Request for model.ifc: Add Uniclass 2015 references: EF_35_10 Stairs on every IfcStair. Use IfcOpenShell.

First a look at what the model holds.

```python
import ifcopenshell

model = ifcopenshell.open("model.ifc")
print(model.schema)
print("classifications:", [c.Name for c in model.by_type("IfcClassification")])
for ifc_class in ("IfcDoor", "IfcRoof", "IfcStair", "IfcWall", "IfcWindow"):
    print(ifc_class, len(model.by_type(ifc_class)))
```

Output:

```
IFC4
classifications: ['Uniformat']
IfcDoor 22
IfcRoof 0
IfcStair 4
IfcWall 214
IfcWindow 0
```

```python
import ifcopenshell
import ifcopenshell.api.classification

model = ifcopenshell.open("model.ifc")

system = ifcopenshell.api.classification.add_classification(model, classification="Uniclass 2015")

codes = {
    "IfcStair": ("EF_35_10", "Stairs"),
}
for ifc_class, (code, name) in codes.items():
    products = model.by_type(ifc_class)
    ifcopenshell.api.classification.add_reference(
        model, products=products, classification=system, identification=code, name=name
    )
    print(code, len(products))

model.write("model_edited.ifc")
```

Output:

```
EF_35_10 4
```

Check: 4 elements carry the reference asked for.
